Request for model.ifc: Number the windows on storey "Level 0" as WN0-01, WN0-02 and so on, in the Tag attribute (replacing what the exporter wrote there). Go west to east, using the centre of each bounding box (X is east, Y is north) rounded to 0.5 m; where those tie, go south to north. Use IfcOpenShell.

First a look at what the model holds.

```python
import ifcopenshell
import ifcopenshell.util.element
import ifcopenshell.util.placement

model = ifcopenshell.open("model.ifc")
print(model.schema)
storey = next(s for s in model.by_type("IfcBuildingStorey") if s.Name == "Level 0")
windows = [e for e in ifcopenshell.util.element.get_decomposition(storey) if e.is_a("IfcWindow")]
for e in sorted(windows, key=lambda e: e.id()):
    origin = ifcopenshell.util.placement.get_local_placement(e.ObjectPlacement)[:3, 3]
    print(e.id(), e.Tag, e.Name, origin.round(2) + 0.0, sep=" | ")
```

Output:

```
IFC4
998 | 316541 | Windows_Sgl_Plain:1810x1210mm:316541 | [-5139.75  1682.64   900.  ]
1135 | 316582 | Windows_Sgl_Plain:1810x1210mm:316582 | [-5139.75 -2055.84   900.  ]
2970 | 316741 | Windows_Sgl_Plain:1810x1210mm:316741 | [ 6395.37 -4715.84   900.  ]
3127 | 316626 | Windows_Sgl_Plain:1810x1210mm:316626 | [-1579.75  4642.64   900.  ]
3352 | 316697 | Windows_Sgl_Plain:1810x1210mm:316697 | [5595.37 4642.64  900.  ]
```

```python
import ifcopenshell
import ifcopenshell.geom
import ifcopenshell.util.element
import ifcopenshell.util.shape

model = ifcopenshell.open("model.ifc")
settings = ifcopenshell.geom.settings()
settings.set("use-world-coords", True)


def centre(element):
    shape = ifcopenshell.geom.create_shape(settings, element)
    return ifcopenshell.util.shape.get_bbox_centroid(shape.geometry)


storey = next(s for s in model.by_type("IfcBuildingStorey") if s.Name == "Level 0")
windows = [e for e in ifcopenshell.util.element.get_decomposition(storey) if e.is_a("IfcWindow")]

# Insertion points can sit at a corner or the storey origin, so sort by the geometry (in metres).
centres = {e: centre(e) for e in windows}
windows.sort(key=lambda e: (round(centres[e][0] / 0.5), centres[e][1]))

for i, e in enumerate(windows, start=1):
    number = f"WN0-{i:02d}"
    e.Tag = number
    print(e.id(), number)

model.write("model_v2.ifc")
```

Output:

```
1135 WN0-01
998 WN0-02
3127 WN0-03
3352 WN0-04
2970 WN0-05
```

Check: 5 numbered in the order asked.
